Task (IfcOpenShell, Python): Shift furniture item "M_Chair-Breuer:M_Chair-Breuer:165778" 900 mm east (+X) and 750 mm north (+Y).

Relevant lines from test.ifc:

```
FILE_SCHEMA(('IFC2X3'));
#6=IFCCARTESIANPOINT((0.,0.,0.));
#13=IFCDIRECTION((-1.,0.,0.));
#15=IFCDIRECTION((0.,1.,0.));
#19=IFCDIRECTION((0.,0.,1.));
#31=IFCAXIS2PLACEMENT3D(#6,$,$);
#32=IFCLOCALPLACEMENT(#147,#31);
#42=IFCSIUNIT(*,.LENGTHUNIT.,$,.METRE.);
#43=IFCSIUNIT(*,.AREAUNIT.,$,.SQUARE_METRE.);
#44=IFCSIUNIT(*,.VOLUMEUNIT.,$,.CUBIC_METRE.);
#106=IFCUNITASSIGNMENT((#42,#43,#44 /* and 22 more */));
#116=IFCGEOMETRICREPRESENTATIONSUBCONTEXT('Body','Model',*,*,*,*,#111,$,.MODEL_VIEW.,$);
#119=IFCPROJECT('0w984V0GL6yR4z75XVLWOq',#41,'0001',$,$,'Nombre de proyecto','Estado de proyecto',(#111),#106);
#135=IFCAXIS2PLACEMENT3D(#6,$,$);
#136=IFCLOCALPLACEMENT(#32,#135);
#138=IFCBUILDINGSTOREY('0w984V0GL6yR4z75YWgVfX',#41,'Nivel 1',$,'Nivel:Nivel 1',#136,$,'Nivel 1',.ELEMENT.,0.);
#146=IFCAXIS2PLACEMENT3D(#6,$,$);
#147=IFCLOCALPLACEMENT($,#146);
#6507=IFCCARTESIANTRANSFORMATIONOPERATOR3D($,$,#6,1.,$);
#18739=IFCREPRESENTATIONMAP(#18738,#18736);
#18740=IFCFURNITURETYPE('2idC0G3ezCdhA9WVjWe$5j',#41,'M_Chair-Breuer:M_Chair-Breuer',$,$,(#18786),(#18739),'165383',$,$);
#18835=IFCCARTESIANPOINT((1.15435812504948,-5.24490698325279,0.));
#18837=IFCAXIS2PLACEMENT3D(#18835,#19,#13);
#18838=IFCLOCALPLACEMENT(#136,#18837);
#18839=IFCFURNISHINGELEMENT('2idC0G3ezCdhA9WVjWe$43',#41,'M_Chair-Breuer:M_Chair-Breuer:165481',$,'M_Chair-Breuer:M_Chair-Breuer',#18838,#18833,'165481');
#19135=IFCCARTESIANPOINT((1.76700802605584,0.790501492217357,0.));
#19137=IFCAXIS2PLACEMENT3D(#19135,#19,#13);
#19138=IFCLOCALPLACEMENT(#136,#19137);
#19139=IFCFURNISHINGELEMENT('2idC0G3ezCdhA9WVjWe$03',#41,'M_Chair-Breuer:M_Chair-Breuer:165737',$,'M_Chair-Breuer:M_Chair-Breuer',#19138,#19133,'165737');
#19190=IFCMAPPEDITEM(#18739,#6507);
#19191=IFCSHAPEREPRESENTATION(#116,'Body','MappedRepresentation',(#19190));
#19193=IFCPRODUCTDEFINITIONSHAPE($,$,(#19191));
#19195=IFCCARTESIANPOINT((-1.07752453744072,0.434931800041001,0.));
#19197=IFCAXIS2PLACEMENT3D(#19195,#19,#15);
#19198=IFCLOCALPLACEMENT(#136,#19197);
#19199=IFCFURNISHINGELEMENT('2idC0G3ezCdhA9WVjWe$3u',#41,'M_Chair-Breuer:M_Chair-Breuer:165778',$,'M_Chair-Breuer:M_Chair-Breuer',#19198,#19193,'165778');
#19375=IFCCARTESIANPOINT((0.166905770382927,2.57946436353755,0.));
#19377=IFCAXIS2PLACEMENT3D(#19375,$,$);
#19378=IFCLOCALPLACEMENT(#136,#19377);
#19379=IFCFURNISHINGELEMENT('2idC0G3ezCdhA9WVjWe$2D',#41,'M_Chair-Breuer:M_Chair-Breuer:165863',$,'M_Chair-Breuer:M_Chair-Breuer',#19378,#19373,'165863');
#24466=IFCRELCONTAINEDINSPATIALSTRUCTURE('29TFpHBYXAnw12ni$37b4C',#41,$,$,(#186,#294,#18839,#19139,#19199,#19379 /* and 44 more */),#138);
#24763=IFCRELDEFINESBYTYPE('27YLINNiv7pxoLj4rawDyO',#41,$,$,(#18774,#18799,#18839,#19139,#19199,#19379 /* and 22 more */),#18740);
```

```python
import ifcopenshell
import ifcopenshell.api.geometry
import ifcopenshell.util.placement
import ifcopenshell.util.unit

model = ifcopenshell.open("test.ifc")
unit_scale = ifcopenshell.util.unit.calculate_unit_scale(model)

item = model.by_guid("2idC0G3ezCdhA9WVjWe$3u")
matrix = ifcopenshell.util.placement.get_local_placement(item.ObjectPlacement)
matrix[0, 3] += 0.9 / unit_scale
matrix[1, 3] += 0.75 / unit_scale
ifcopenshell.api.geometry.edit_object_placement(model, product=item, matrix=matrix, is_si=False)

print(ifcopenshell.util.placement.get_local_placement(item.ObjectPlacement).round(3) + 0.0)

model.write("test_rev.ifc")
```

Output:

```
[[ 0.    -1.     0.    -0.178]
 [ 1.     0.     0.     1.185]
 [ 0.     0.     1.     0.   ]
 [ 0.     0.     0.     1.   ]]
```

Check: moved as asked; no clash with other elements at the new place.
